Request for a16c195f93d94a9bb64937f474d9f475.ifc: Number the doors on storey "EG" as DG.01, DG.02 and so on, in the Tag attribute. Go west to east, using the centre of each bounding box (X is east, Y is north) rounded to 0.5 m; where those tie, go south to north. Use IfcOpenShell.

First a look at what the model holds.

```python
import ifcopenshell
import ifcopenshell.util.element
import ifcopenshell.util.placement

model = ifcopenshell.open("a16c195f93d94a9bb64937f474d9f475.ifc")
print(model.schema)
storey = next(s for s in model.by_type("IfcBuildingStorey") if s.Name == "EG")
doors = [e for e in ifcopenshell.util.element.get_decomposition(storey) if e.is_a("IfcDoor")]
for e in sorted(doors, key=lambda e: e.id()):
    origin = ifcopenshell.util.placement.get_local_placement(e.ObjectPlacement)[:3, 3]
    print(e.id(), e.Tag, e.Name, origin.round(2) + 0.0, sep=" | ")
```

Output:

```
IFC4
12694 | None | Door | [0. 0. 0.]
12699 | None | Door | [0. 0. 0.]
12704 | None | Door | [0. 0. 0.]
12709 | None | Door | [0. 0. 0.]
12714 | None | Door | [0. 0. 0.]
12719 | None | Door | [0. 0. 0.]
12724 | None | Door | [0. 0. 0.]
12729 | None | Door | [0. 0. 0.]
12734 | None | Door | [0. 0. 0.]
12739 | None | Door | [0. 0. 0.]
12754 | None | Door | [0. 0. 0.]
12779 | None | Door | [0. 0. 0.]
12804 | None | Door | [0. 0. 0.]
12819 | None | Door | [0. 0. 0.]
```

```python
import ifcopenshell
import ifcopenshell.geom
import ifcopenshell.util.element
import ifcopenshell.util.shape

model = ifcopenshell.open("a16c195f93d94a9bb64937f474d9f475.ifc")
settings = ifcopenshell.geom.settings()
settings.set("use-world-coords", True)


def centre(element):
    shape = ifcopenshell.geom.create_shape(settings, element)
    return ifcopenshell.util.shape.get_bbox_centroid(shape.geometry)


storey = next(s for s in model.by_type("IfcBuildingStorey") if s.Name == "EG")
doors = [e for e in ifcopenshell.util.element.get_decomposition(storey) if e.is_a("IfcDoor")]

# Insertion points can sit at a corner or the storey origin, so sort by the geometry (in metres).
centres = {e: centre(e) for e in doors}
doors.sort(key=lambda e: (round(centres[e][0] / 0.5), centres[e][1]))

for i, e in enumerate(doors, start=1):
    number = f"DG.{i:02d}"
    e.Tag = number
    print(e.id(), number)

model.write("a16c195f93d94a9bb64937f474d9f475-out.ifc")
```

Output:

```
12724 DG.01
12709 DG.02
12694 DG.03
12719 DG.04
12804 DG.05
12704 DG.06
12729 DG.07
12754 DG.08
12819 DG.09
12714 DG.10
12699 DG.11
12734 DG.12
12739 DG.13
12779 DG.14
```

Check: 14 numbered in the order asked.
